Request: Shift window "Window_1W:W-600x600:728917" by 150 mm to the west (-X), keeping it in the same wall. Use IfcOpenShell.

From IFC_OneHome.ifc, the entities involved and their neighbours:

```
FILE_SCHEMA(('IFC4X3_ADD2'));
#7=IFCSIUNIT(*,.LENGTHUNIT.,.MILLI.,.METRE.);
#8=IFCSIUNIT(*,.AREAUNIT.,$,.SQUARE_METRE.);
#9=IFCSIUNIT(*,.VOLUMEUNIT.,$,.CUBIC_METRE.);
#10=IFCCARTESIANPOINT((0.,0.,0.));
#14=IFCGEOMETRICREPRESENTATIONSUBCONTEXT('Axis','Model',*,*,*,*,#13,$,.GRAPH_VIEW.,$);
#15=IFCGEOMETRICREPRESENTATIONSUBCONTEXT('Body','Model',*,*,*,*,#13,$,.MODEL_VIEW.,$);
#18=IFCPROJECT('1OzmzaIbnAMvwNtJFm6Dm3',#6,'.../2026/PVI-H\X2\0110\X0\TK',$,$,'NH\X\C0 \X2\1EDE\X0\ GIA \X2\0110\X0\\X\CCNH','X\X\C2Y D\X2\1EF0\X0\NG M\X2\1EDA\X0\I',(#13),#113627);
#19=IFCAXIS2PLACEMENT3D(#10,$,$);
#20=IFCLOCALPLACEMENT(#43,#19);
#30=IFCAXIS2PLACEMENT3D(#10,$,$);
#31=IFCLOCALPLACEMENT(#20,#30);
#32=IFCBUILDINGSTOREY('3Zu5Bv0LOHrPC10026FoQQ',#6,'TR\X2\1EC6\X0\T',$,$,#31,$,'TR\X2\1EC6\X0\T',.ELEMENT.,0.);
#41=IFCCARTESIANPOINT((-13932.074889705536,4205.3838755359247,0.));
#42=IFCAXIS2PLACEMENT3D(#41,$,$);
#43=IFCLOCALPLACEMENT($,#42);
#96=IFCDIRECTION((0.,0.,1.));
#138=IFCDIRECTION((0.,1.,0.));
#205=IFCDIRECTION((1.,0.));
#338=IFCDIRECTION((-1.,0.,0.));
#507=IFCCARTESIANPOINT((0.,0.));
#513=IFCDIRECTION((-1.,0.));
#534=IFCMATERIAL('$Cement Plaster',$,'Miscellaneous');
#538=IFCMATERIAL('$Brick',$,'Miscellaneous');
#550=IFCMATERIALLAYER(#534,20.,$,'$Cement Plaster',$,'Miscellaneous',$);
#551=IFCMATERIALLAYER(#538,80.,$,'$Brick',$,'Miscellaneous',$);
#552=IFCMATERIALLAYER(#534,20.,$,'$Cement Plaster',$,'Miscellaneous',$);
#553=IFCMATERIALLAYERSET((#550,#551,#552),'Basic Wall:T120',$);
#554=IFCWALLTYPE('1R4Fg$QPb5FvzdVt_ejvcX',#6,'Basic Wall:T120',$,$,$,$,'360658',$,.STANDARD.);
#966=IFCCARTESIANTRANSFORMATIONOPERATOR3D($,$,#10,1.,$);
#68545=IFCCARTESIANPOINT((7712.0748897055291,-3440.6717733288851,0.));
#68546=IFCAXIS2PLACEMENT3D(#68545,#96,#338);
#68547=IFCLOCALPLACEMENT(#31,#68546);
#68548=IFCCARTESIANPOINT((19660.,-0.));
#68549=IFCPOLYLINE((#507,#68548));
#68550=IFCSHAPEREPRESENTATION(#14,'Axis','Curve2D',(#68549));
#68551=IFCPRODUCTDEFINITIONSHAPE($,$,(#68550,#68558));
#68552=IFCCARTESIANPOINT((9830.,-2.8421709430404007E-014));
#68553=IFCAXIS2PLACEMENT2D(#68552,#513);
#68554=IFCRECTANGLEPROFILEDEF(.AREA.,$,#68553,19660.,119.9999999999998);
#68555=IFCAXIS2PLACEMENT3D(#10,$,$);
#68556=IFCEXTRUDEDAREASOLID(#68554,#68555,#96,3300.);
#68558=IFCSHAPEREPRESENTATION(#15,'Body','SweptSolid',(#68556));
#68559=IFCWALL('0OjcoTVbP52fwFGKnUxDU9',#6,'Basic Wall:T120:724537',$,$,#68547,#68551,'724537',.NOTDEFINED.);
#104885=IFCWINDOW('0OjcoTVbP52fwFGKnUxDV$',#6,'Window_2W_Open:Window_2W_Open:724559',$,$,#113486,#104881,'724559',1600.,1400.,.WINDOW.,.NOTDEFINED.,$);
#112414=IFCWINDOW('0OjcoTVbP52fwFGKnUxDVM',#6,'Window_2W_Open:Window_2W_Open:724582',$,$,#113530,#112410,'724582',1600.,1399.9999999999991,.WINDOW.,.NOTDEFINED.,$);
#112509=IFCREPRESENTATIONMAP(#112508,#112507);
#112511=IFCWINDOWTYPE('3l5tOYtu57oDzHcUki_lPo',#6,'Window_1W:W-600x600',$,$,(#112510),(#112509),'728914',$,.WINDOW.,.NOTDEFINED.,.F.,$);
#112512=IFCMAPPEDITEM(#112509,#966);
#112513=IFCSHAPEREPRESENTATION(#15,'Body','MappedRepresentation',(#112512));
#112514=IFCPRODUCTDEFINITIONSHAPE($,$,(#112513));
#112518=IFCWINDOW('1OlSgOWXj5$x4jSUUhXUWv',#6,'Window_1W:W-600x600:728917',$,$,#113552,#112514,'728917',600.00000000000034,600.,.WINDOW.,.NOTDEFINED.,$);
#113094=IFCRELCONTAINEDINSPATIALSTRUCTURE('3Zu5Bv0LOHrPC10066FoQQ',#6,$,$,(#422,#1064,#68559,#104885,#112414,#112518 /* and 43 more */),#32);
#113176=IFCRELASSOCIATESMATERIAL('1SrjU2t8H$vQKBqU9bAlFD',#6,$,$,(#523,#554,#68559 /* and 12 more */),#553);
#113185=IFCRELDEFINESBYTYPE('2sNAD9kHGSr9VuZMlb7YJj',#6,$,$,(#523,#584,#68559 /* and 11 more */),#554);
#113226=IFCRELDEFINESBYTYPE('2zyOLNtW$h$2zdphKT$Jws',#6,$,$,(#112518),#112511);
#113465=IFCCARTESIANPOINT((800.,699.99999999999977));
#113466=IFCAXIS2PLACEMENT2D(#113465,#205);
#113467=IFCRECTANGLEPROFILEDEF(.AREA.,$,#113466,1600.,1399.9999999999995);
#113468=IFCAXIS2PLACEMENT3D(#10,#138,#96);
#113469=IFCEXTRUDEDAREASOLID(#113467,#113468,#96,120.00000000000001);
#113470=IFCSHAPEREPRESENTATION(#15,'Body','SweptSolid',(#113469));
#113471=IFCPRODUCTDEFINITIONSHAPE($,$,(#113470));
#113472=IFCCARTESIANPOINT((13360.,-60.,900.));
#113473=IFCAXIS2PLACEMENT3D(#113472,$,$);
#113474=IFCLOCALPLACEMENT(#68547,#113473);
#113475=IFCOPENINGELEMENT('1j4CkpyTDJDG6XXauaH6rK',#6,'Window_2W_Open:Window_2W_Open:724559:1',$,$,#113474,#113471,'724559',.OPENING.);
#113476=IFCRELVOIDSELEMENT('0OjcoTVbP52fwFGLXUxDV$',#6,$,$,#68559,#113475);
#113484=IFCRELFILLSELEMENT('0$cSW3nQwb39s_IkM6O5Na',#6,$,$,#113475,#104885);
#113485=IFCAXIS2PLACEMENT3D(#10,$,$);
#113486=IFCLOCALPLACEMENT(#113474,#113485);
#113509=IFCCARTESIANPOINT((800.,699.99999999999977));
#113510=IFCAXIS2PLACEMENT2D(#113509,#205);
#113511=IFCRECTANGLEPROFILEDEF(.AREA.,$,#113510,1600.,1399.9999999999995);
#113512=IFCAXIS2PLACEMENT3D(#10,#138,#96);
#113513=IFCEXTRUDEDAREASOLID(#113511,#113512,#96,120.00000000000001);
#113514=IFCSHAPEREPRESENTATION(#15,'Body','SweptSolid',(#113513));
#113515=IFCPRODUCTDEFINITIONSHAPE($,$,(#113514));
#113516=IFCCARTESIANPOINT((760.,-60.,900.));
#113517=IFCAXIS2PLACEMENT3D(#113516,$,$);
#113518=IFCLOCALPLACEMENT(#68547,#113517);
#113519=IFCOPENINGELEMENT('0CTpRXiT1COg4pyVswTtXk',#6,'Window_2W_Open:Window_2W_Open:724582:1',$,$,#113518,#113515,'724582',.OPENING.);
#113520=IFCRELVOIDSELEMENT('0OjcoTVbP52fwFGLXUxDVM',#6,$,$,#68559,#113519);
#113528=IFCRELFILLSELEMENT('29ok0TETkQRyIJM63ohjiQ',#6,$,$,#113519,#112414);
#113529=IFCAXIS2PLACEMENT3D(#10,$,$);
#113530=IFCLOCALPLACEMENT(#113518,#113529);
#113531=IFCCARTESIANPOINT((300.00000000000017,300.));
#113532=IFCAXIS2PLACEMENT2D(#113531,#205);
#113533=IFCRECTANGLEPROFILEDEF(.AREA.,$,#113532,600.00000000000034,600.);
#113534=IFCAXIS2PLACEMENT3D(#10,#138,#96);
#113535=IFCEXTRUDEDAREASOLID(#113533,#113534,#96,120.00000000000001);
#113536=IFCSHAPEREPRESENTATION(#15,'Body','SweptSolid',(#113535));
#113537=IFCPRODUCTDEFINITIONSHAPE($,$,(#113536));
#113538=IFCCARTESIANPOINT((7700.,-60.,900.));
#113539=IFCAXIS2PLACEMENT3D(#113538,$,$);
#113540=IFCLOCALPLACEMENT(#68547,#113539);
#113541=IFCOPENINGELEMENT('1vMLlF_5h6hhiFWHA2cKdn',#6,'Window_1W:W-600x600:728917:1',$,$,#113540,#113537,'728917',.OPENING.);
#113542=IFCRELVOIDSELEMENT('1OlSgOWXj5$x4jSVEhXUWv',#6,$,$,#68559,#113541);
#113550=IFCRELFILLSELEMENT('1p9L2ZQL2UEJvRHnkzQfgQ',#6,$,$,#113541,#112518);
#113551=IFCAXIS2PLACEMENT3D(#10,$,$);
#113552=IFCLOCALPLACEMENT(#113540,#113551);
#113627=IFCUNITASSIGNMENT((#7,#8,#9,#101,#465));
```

```python
import ifcopenshell
import ifcopenshell.api.geometry
import ifcopenshell.util.placement
import ifcopenshell.util.unit

model = ifcopenshell.open("IFC_OneHome.ifc")
unit_scale = ifcopenshell.util.unit.calculate_unit_scale(model)

window = model.by_guid("1OlSgOWXj5$x4jSUUhXUWv")
opening = window.FillsVoids[0].RelatingOpeningElement
wall = opening.VoidsElements[0].RelatingBuildingElement

wall_matrix = ifcopenshell.util.placement.get_local_placement(wall.ObjectPlacement)
shift = wall_matrix[:3, 0] * 0.15 / unit_scale
before = ifcopenshell.util.placement.get_local_placement(window.ObjectPlacement)[:3, 3].copy()

# The window is placed relative to its opening, so it follows when the opening moves.
matrix = ifcopenshell.util.placement.get_local_placement(opening.ObjectPlacement)
matrix[:3, 3] += shift
ifcopenshell.api.geometry.edit_object_placement(
    model, product=opening, matrix=matrix, is_si=False, should_transform_children=True
)

after = ifcopenshell.util.placement.get_local_placement(window.ObjectPlacement)[:3, 3]
print("window moved by", (after - before).round(3) + 0.0)

model.write("IFC_OneHome_updated.ifc")
```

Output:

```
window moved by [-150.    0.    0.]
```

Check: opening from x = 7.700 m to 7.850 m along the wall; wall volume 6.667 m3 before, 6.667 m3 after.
